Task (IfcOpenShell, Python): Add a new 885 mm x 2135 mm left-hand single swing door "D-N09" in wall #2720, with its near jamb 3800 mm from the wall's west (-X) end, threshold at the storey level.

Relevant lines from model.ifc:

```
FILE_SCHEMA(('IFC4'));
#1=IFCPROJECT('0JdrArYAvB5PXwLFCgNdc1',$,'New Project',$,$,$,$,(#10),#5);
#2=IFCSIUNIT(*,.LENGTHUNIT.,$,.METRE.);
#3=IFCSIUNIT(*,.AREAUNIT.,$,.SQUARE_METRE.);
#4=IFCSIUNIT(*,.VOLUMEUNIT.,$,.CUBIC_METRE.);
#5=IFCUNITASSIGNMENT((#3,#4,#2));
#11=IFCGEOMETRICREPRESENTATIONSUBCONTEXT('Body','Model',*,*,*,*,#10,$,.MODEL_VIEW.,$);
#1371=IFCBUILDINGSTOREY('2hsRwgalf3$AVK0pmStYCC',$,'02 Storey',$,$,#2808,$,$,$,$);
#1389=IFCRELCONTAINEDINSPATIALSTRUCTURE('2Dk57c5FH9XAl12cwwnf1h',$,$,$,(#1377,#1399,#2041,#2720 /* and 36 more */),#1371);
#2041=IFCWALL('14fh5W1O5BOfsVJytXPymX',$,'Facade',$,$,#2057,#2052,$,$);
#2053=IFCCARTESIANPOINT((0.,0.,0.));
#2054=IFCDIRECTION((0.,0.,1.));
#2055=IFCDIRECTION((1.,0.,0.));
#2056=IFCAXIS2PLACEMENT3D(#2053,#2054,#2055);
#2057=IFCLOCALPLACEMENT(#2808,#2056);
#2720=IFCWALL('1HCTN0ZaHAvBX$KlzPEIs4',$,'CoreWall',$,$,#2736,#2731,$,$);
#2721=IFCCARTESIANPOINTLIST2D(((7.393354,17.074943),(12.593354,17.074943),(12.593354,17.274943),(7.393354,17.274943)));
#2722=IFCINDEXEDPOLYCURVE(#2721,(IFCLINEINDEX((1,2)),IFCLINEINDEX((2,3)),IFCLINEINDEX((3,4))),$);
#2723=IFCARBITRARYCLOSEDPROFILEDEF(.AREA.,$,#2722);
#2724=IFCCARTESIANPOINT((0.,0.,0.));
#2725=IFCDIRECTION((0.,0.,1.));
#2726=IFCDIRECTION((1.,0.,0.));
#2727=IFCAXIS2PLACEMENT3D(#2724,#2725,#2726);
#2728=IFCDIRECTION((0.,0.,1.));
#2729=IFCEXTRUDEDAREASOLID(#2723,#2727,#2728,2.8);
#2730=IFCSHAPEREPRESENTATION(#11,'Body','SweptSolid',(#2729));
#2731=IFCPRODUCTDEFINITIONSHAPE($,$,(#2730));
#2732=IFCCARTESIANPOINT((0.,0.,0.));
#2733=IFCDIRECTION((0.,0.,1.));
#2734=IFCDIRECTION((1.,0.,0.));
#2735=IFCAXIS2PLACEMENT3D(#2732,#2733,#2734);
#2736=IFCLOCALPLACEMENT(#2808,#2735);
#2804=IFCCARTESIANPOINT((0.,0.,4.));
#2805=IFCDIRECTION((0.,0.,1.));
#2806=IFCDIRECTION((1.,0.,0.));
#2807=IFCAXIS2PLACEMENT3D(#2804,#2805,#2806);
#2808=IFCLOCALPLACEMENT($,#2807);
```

```python
import numpy as np
import ifcopenshell
import ifcopenshell.api.feature
import ifcopenshell.api.geometry
import ifcopenshell.api.root
import ifcopenshell.api.spatial
import ifcopenshell.geom
import ifcopenshell.util.element
import ifcopenshell.util.placement
import ifcopenshell.util.representation
import ifcopenshell.util.shape
import ifcopenshell.util.unit

model = ifcopenshell.open("model.ifc")
unit_scale = ifcopenshell.util.unit.calculate_unit_scale(model)
settings = ifcopenshell.geom.settings()


def volume(element):
    """Net volume in cubic metres, openings subtracted."""
    shape = ifcopenshell.geom.create_shape(settings, element)
    return ifcopenshell.util.shape.get_volume(shape.geometry)


wall = model.by_guid("1HCTN0ZaHAvBX$KlzPEIs4")
storey = ifcopenshell.util.element.get_container(wall, ifc_class="IfcBuildingStorey")
context = ifcopenshell.util.representation.get_context(model, "Model", "Body", "MODEL_VIEW")
before = volume(wall)

width, height, from_end, sill = 0.885, 2.135, 3.8, 0.0  # metres

# The wall runs along its own X axis, and the end named is its -X end.
wall_shape = ifcopenshell.geom.create_shape(settings, wall)
x, y, z = ifcopenshell.util.shape.get_vertices(wall_shape.geometry).T
start = x.min() + from_end
face, thickness = float(y.min()), float(y.max() - y.min())
wall_matrix = ifcopenshell.util.placement.get_local_placement(wall.ObjectPlacement)
level = ifcopenshell.util.placement.get_local_placement(storey.ObjectPlacement)[2, 3]


def in_wall(x, y):
    """Placement at x, y metres in the wall's axes, at sill height."""
    matrix = wall_matrix.copy()
    matrix[:, 3] = wall_matrix @ np.array([x / unit_scale, y / unit_scale, 0.0, 1.0])
    matrix[2, 3] = level + sill / unit_scale
    return matrix


# Opening: a box that overshoots both wall faces by 50 mm.
opening = ifcopenshell.api.root.create_entity(model, ifc_class="IfcOpeningElement", predefined_type="OPENING")
box = ifcopenshell.api.geometry.add_wall_representation(
    model, context=context, length=width, height=height, thickness=thickness + 0.1
)
ifcopenshell.api.geometry.assign_representation(model, product=opening, representation=box)
ifcopenshell.api.geometry.edit_object_placement(model, product=opening, matrix=in_wall(start, face - 0.05), is_si=False)
ifcopenshell.api.feature.add_feature(model, feature=opening, element=wall)

door = ifcopenshell.api.root.create_entity(model, ifc_class="IfcDoor", name="D-N09", predefined_type="DOOR")
door.OverallWidth, door.OverallHeight = width / unit_scale, height / unit_scale
door.OperationType = "SINGLE_SWING_LEFT"
body = ifcopenshell.api.geometry.add_door_representation(
    model,
    context=context,
    overall_width=door.OverallWidth,
    overall_height=door.OverallHeight,
    operation_type="SINGLE_SWING_LEFT",
    lining_properties={"LiningDepth": thickness / unit_scale, "ThresholdDepth": thickness / unit_scale},
)
ifcopenshell.api.geometry.assign_representation(model, product=door, representation=body)
ifcopenshell.api.spatial.assign_container(model, products=[door], relating_structure=storey)
ifcopenshell.api.feature.add_filling(model, opening=opening, element=door)

# The lining spans the wall, so the door starts at the wall face.
ifcopenshell.api.geometry.edit_object_placement(model, product=door, matrix=in_wall(start, face), is_si=False)

after = volume(wall)

print(f"wall volume {before:.3f} -> {after:.3f} m3")

model.write("model-out.ifc")
```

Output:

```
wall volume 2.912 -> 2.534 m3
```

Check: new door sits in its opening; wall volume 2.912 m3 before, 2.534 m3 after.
